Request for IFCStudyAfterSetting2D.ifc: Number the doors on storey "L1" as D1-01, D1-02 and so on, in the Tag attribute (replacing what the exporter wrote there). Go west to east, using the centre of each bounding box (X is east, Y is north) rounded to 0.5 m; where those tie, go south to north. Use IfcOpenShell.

First a look at what the model holds.

```python
import ifcopenshell
import ifcopenshell.util.element
import ifcopenshell.util.placement

model = ifcopenshell.open("IFCStudyAfterSetting2D.ifc")
print(model.schema)
storey = next(s for s in model.by_type("IfcBuildingStorey") if s.Name == "L1")
doors = [e for e in ifcopenshell.util.element.get_decomposition(storey) if e.is_a("IfcDoor")]
for e in sorted(doors, key=lambda e: e.id()):
    origin = ifcopenshell.util.placement.get_local_placement(e.ObjectPlacement)[:3, 3]
    print(e.id(), e.Tag, e.Name, origin.round(2) + 0.0, sep=" | ")
```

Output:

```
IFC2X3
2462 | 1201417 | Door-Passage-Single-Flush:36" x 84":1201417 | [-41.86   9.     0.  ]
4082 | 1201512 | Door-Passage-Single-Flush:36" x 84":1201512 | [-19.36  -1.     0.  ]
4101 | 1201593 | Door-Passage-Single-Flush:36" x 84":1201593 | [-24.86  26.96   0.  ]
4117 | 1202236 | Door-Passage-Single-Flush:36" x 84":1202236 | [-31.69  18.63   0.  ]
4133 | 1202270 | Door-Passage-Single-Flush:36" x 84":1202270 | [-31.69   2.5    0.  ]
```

```python
import ifcopenshell
import ifcopenshell.geom
import ifcopenshell.util.element
import ifcopenshell.util.shape

model = ifcopenshell.open("IFCStudyAfterSetting2D.ifc")
settings = ifcopenshell.geom.settings()
settings.set("use-world-coords", True)


def centre(element):
    shape = ifcopenshell.geom.create_shape(settings, element)
    return ifcopenshell.util.shape.get_bbox_centroid(shape.geometry)


storey = next(s for s in model.by_type("IfcBuildingStorey") if s.Name == "L1")
doors = [e for e in ifcopenshell.util.element.get_decomposition(storey) if e.is_a("IfcDoor")]

# Insertion points can sit at a corner or the storey origin, so sort by the geometry (in metres).
centres = {e: centre(e) for e in doors}
doors.sort(key=lambda e: (round(centres[e][0] / 0.5), centres[e][1]))

for i, e in enumerate(doors, start=1):
    number = f"D1-{i:02d}"
    e.Tag = number
    print(e.id(), number)

model.write("IFCStudyAfterSetting2D_edited.ifc")
```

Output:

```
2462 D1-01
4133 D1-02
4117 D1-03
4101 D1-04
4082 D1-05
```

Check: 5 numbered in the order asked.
